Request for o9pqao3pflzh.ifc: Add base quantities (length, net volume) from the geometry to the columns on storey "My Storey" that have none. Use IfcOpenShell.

First a look at what the model holds.

```python
import ifcopenshell
import ifcopenshell.util.element
import ifcopenshell.util.unit

model = ifcopenshell.open("o9pqao3pflzh.ifc")
print(model.schema)
for unit_type in ("LENGTHUNIT", "AREAUNIT", "VOLUMEUNIT"):
    print(unit_type, ifcopenshell.util.unit.calculate_unit_scale(model, unit_type))
storey = next(s for s in model.by_type("IfcBuildingStorey") if s.Name == "My Storey")
columns = [e for e in ifcopenshell.util.element.get_decomposition(storey) if e.is_a("IfcColumn")]
for e in sorted(columns, key=lambda e: e.id()):
    print(e.id(), e.is_a(), e.Name, list(ifcopenshell.util.element.get_psets(e, qtos_only=True)), sep=" | ")
```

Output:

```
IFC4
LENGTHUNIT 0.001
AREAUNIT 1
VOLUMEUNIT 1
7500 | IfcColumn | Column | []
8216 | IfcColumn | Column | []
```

```python
import ifcopenshell
import ifcopenshell.api.pset
import ifcopenshell.geom
import ifcopenshell.util.element
import ifcopenshell.util.shape
import ifcopenshell.util.unit

model = ifcopenshell.open("o9pqao3pflzh.ifc")
unit_scale = ifcopenshell.util.unit.calculate_unit_scale(model)
volume_scale = ifcopenshell.util.unit.calculate_unit_scale(model, "VOLUMEUNIT")
settings = ifcopenshell.geom.settings()

storey = next(s for s in model.by_type("IfcBuildingStorey") if s.Name == "My Storey")
columns = [e for e in ifcopenshell.util.element.get_decomposition(storey) if e.is_a("IfcColumn")]

for e in sorted(columns, key=lambda e: e.id()):
    if ifcopenshell.util.element.get_psets(e, qtos_only=True, should_inherit=False):
        continue
    # Geometry comes back in metres, in the element's own axes.
    shape = ifcopenshell.geom.create_shape(settings, e)
    values = {
        "Length": ifcopenshell.util.shape.get_z(shape.geometry) / unit_scale,
        "NetVolume": ifcopenshell.util.shape.get_volume(shape.geometry) / volume_scale,
    }
    qto = ifcopenshell.api.pset.add_qto(model, product=e, name="Qto_ColumnBaseQuantities")
    ifcopenshell.api.pset.edit_qto(model, qto=qto, properties=values)
    print(e.id(), {k: round(v, 3) for k, v in values.items()})

model.write("o9pqao3pflzh-out.ifc")
```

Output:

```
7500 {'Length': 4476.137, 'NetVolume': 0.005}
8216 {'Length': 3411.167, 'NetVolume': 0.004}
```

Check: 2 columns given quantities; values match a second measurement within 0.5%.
